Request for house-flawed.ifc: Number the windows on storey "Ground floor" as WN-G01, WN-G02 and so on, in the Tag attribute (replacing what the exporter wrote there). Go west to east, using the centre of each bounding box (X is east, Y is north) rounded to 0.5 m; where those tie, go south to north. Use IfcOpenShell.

First a look at what the model holds.

```python
import ifcopenshell
import ifcopenshell.util.element
import ifcopenshell.util.placement

model = ifcopenshell.open("house-flawed.ifc")
print(model.schema)
storey = next(s for s in model.by_type("IfcBuildingStorey") if s.Name == "Ground floor")
windows = [e for e in ifcopenshell.util.element.get_decomposition(storey) if e.is_a("IfcWindow")]
for e in sorted(windows, key=lambda e: e.id()):
    origin = ifcopenshell.util.placement.get_local_placement(e.ObjectPlacement)[:3, 3]
    print(e.id(), e.Tag, e.Name, origin.round(2) + 0.0, sep=" | ")
```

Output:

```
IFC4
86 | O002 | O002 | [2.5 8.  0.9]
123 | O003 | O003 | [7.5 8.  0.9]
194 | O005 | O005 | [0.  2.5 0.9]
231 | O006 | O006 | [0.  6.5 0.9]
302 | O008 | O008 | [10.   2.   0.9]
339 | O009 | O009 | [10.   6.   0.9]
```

```python
import ifcopenshell
import ifcopenshell.geom
import ifcopenshell.util.element
import ifcopenshell.util.shape

model = ifcopenshell.open("house-flawed.ifc")
settings = ifcopenshell.geom.settings()
settings.set("use-world-coords", True)


def centre(element):
    shape = ifcopenshell.geom.create_shape(settings, element)
    return ifcopenshell.util.shape.get_bbox_centroid(shape.geometry)


storey = next(s for s in model.by_type("IfcBuildingStorey") if s.Name == "Ground floor")
windows = [e for e in ifcopenshell.util.element.get_decomposition(storey) if e.is_a("IfcWindow")]

# Insertion points can sit at a corner or the storey origin, so sort by the geometry (in metres).
centres = {e: centre(e) for e in windows}
windows.sort(key=lambda e: (round(centres[e][0] / 0.5), centres[e][1]))

for i, e in enumerate(windows, start=1):
    number = f"WN-G{i:02d}"
    e.Tag = number
    print(e.id(), number)

model.write("house-flawed-out.ifc")
```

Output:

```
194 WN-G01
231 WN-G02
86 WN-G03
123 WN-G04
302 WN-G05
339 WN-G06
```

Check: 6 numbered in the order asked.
